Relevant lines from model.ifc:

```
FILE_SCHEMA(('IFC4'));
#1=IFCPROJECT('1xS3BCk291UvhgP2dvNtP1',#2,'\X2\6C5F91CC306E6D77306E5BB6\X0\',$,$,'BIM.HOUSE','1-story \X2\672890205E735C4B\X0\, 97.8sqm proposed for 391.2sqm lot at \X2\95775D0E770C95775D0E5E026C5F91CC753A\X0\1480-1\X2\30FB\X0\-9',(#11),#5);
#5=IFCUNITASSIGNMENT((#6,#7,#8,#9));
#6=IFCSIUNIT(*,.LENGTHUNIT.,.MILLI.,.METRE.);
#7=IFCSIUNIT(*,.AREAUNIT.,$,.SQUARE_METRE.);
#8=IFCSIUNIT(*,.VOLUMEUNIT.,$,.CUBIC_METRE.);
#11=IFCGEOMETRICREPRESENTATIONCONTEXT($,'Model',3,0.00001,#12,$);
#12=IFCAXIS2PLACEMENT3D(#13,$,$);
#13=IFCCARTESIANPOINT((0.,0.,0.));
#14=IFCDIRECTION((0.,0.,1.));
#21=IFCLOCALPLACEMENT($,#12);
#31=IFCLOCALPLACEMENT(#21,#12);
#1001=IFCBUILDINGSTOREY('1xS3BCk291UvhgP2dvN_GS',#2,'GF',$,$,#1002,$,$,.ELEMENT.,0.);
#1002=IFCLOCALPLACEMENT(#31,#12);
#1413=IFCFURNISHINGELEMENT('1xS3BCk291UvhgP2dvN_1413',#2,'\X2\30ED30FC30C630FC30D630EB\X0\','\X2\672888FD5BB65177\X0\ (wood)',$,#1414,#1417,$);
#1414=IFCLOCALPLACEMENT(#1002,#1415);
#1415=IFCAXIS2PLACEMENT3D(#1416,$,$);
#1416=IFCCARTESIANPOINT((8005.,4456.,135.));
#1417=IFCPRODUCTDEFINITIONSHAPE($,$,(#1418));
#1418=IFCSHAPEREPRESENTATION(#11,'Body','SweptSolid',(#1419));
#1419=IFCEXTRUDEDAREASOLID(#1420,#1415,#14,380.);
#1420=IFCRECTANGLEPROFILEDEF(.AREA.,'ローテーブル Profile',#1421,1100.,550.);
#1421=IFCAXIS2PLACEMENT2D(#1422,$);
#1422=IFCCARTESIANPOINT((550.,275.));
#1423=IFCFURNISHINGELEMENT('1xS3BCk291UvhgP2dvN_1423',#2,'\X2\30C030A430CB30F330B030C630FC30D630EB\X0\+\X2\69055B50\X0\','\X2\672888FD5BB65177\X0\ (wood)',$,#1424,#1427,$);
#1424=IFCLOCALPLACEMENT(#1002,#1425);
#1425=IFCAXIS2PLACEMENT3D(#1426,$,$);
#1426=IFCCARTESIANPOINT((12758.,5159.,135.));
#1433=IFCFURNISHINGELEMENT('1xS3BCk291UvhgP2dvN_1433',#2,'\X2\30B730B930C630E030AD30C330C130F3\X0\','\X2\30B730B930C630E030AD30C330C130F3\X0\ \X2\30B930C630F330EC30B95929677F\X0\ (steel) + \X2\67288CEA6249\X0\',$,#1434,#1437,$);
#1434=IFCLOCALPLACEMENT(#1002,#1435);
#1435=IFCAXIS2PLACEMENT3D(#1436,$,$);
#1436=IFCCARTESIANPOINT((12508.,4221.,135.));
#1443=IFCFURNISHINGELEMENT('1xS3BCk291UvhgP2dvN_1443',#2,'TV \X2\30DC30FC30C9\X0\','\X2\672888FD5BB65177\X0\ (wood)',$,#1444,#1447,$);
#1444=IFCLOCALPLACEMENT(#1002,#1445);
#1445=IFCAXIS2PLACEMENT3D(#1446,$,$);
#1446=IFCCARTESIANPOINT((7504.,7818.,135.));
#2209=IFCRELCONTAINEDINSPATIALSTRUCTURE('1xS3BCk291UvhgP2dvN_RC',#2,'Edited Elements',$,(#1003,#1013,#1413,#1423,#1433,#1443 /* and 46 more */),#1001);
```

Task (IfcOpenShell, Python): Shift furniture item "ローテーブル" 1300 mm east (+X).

```python
import ifcopenshell
import ifcopenshell.api.geometry
import ifcopenshell.util.placement
import ifcopenshell.util.unit

model = ifcopenshell.open("model.ifc")
unit_scale = ifcopenshell.util.unit.calculate_unit_scale(model)

item = model.by_guid("1xS3BCk291UvhgP2dvN_1413")
matrix = ifcopenshell.util.placement.get_local_placement(item.ObjectPlacement)
matrix[0, 3] += 1.3 / unit_scale
ifcopenshell.api.geometry.edit_object_placement(model, product=item, matrix=matrix, is_si=False)

print(ifcopenshell.util.placement.get_local_placement(item.ObjectPlacement).round(3) + 0.0)

model.write("model_updated.ifc")
```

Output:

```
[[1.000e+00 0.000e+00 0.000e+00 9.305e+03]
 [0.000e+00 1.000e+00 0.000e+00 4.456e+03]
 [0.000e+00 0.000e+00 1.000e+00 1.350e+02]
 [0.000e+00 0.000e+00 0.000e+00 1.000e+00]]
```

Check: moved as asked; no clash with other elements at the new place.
